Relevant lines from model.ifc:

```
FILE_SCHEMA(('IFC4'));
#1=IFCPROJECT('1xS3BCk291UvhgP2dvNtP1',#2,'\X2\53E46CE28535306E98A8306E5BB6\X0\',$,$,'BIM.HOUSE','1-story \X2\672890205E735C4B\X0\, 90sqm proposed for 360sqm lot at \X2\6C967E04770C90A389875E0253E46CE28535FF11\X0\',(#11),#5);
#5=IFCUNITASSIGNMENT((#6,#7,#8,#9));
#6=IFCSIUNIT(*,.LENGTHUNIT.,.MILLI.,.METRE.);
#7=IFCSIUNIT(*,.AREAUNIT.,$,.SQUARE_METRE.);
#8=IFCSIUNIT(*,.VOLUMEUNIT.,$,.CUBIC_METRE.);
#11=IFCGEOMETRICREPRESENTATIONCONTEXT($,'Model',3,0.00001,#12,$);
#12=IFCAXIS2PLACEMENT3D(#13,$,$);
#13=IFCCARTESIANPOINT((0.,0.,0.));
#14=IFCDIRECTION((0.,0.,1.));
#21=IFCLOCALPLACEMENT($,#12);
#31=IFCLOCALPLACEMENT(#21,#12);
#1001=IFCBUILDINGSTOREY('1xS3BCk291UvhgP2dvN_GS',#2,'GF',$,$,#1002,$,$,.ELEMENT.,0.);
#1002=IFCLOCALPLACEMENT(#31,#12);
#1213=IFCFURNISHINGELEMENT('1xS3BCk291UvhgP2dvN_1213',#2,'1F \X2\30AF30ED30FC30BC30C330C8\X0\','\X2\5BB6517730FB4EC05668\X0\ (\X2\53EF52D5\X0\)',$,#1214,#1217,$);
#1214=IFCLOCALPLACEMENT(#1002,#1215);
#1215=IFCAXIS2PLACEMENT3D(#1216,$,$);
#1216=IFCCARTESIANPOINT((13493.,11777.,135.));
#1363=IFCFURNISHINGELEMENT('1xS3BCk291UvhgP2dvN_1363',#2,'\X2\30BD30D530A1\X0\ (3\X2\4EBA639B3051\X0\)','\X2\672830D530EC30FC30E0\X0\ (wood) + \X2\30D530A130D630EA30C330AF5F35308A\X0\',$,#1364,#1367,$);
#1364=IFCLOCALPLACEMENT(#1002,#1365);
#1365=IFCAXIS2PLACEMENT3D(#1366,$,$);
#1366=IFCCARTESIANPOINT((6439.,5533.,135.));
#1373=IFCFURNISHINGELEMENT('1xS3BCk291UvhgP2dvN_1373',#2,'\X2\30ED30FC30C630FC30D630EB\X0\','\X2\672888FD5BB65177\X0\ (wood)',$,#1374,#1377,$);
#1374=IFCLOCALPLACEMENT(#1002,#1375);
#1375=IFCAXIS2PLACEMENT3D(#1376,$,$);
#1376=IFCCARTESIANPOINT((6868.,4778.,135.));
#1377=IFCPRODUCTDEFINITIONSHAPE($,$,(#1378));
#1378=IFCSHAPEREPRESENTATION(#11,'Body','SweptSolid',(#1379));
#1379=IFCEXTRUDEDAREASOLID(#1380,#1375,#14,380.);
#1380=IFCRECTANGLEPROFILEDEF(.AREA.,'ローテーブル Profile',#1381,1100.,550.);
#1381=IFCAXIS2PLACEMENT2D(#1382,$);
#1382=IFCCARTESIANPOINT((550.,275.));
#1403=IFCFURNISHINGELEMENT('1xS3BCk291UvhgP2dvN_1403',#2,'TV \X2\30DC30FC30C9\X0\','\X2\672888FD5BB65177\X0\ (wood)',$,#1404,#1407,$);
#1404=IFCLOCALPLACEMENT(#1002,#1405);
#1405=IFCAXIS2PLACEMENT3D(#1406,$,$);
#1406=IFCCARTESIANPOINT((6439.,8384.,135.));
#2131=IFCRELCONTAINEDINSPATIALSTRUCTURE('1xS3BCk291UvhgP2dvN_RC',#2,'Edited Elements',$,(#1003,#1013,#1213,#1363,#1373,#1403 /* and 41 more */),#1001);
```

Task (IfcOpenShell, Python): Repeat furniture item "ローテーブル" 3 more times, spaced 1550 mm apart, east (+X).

```python
import numpy as np
import ifcopenshell
import ifcopenshell.api.geometry
import ifcopenshell.api.root
import ifcopenshell.util.element
import ifcopenshell.util.placement

model = ifcopenshell.open("model.ifc")


def reuse_history(source, copy):
    """copy_class also copies each property set's owner history, people and application; keep the originals."""
    for rel in copy.IsDefinedBy:
        if rel.is_a("IfcRelDefinesByProperties") and (history := rel.RelatingPropertyDefinition.OwnerHistory):
            rel.RelatingPropertyDefinition.OwnerHistory = source.OwnerHistory
            ifcopenshell.util.element.remove_deep2(model, history)


source = model.by_id(1373)
base = ifcopenshell.util.placement.get_local_placement(source.ObjectPlacement)
step = np.array([1.0, 0.0, 0.0]) * 1550.0

for i in range(1, 4):
    copy = ifcopenshell.api.root.copy_class(model, product=source)
    copy.Representation = ifcopenshell.util.element.copy_deep(
        model, source.Representation, exclude=["IfcGeometricRepresentationContext", "IfcRepresentationMap"]
    )
    reuse_history(source, copy)
    matrix = base.copy()
    matrix[:3, 3] += i * step
    print("added at", matrix[:3, 3].round(3) + 0.0)
    ifcopenshell.api.geometry.edit_object_placement(model, product=copy, matrix=matrix, is_si=False)

model.write("model_v2.ifc")
```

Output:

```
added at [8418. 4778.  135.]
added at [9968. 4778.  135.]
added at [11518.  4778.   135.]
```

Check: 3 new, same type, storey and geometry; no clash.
